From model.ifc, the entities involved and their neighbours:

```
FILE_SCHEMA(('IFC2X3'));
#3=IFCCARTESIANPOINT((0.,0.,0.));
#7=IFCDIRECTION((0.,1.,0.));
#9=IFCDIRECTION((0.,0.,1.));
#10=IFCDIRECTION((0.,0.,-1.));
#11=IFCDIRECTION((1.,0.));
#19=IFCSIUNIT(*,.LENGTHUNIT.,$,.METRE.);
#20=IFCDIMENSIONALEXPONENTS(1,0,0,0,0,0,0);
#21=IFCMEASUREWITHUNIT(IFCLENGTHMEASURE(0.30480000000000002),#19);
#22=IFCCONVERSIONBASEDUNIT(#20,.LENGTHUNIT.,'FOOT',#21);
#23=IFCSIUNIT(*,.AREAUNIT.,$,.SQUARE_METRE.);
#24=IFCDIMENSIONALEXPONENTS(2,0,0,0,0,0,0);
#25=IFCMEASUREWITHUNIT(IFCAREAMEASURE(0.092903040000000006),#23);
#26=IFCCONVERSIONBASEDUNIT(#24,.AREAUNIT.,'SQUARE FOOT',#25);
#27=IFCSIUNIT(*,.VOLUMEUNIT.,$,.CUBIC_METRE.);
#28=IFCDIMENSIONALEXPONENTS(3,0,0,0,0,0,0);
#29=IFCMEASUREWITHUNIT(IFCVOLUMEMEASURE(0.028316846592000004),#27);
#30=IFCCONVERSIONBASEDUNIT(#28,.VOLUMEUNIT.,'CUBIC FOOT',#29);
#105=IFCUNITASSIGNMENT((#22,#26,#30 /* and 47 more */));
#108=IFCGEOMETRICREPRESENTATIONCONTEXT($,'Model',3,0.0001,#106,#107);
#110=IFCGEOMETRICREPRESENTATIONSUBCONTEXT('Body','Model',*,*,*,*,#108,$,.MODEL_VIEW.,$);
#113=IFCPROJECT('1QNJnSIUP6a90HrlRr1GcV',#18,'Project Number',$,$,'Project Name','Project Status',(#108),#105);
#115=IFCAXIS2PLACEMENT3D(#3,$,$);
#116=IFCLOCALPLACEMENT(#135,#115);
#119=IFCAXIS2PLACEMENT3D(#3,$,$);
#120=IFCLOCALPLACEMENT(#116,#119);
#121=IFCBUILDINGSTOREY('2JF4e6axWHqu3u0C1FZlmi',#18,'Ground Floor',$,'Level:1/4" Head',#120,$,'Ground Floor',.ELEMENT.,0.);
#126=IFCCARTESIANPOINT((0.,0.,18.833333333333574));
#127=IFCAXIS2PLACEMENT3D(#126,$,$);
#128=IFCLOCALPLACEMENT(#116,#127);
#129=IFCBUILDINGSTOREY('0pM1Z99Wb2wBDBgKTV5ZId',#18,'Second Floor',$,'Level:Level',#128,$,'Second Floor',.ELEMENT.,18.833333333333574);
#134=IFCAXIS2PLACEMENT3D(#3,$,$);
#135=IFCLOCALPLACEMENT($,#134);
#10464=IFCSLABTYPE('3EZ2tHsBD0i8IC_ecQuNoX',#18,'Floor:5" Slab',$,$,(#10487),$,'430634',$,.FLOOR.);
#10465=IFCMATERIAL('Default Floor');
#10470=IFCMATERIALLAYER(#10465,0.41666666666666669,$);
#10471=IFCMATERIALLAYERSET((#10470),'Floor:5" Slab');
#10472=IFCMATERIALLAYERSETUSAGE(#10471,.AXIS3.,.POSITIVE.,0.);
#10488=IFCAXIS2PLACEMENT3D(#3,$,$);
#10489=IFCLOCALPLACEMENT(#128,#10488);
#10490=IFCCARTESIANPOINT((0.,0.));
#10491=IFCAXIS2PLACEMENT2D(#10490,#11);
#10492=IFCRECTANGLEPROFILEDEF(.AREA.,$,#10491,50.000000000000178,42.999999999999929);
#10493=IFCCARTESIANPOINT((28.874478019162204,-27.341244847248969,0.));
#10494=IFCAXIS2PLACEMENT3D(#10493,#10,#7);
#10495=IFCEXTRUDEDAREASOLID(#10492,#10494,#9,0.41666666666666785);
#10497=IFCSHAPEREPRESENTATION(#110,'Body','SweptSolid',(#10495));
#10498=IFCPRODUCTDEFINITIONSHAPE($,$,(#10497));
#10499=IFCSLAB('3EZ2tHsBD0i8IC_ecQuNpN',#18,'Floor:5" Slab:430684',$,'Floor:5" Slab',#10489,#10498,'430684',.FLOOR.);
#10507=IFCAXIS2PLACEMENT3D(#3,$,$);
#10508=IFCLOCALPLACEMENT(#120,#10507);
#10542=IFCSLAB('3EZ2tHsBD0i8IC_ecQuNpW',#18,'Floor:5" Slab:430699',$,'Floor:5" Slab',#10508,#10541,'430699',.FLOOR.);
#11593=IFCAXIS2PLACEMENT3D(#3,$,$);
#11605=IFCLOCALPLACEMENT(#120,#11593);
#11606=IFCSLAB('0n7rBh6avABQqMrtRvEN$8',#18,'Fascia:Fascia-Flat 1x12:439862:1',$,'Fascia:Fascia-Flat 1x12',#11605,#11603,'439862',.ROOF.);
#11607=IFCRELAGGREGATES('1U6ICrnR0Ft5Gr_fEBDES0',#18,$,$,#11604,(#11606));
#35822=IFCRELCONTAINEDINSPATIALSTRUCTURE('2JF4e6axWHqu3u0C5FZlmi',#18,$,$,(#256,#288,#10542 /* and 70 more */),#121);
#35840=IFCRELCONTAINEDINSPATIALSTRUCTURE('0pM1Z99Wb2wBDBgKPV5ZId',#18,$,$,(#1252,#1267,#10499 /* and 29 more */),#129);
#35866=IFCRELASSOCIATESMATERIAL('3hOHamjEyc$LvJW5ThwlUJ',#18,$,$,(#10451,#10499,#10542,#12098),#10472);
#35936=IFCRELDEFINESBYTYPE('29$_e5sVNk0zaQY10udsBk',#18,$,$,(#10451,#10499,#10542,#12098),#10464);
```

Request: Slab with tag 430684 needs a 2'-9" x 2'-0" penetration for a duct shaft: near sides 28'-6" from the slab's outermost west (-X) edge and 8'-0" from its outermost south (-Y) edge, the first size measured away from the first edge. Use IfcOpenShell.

```python
import numpy as np
import ifcopenshell
import ifcopenshell.api.feature
import ifcopenshell.api.geometry
import ifcopenshell.api.root
import ifcopenshell.geom
import ifcopenshell.util.placement
import ifcopenshell.util.representation
import ifcopenshell.util.shape
import ifcopenshell.util.unit

model = ifcopenshell.open("model.ifc")
unit_scale = ifcopenshell.util.unit.calculate_unit_scale(model)
settings = ifcopenshell.geom.settings()


def volume(element):
    """Net volume in cubic metres, openings subtracted."""
    shape = ifcopenshell.geom.create_shape(settings, element)
    return ifcopenshell.util.shape.get_volume(shape.geometry)


slab = model.by_guid("3EZ2tHsBD0i8IC_ecQuNpN")
before = volume(slab)

# Extent in the slab's own axes, in metres. The edges named are its -X and -Y sides.
slab_shape = ifcopenshell.geom.create_shape(settings, slab)
vertices = ifcopenshell.util.shape.get_vertices(slab_shape.geometry)
x_min, y_min, bottom = vertices.min(axis=0)
top = vertices[:, 2].max()

opening = ifcopenshell.api.root.create_entity(model, ifc_class="IfcOpeningElement", name="Duct shaft opening")
context = ifcopenshell.util.representation.get_context(model, "Model", "Body", "MODEL_VIEW")
width, depth = 0.8382, 0.6096
outline = [(0.0, 0.0), (width, 0.0), (width, depth), (0.0, depth), (0.0, 0.0)]
# Overshoot both faces by 50 mm so the cut is clean.
shape = ifcopenshell.api.geometry.add_slab_representation(
    model, context=context, depth=top - bottom + 0.1, polyline=outline
)
ifcopenshell.api.geometry.assign_representation(model, product=opening, representation=shape)

matrix = ifcopenshell.util.placement.get_local_placement(slab.ObjectPlacement)
matrix[:, 3] = matrix @ np.append(np.array([x_min + 8.6868, y_min + 2.4384, bottom - 0.05]) / unit_scale, 1.0)
ifcopenshell.api.geometry.edit_object_placement(model, product=opening, matrix=matrix, is_si=False)
ifcopenshell.api.feature.add_feature(model, feature=opening, element=slab)

after = volume(slab)

print(f"slab volume {before:.3f} -> {after:.3f} m3")

model.write("model-out.ifc")
```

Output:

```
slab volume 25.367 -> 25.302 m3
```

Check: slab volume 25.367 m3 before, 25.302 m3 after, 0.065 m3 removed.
